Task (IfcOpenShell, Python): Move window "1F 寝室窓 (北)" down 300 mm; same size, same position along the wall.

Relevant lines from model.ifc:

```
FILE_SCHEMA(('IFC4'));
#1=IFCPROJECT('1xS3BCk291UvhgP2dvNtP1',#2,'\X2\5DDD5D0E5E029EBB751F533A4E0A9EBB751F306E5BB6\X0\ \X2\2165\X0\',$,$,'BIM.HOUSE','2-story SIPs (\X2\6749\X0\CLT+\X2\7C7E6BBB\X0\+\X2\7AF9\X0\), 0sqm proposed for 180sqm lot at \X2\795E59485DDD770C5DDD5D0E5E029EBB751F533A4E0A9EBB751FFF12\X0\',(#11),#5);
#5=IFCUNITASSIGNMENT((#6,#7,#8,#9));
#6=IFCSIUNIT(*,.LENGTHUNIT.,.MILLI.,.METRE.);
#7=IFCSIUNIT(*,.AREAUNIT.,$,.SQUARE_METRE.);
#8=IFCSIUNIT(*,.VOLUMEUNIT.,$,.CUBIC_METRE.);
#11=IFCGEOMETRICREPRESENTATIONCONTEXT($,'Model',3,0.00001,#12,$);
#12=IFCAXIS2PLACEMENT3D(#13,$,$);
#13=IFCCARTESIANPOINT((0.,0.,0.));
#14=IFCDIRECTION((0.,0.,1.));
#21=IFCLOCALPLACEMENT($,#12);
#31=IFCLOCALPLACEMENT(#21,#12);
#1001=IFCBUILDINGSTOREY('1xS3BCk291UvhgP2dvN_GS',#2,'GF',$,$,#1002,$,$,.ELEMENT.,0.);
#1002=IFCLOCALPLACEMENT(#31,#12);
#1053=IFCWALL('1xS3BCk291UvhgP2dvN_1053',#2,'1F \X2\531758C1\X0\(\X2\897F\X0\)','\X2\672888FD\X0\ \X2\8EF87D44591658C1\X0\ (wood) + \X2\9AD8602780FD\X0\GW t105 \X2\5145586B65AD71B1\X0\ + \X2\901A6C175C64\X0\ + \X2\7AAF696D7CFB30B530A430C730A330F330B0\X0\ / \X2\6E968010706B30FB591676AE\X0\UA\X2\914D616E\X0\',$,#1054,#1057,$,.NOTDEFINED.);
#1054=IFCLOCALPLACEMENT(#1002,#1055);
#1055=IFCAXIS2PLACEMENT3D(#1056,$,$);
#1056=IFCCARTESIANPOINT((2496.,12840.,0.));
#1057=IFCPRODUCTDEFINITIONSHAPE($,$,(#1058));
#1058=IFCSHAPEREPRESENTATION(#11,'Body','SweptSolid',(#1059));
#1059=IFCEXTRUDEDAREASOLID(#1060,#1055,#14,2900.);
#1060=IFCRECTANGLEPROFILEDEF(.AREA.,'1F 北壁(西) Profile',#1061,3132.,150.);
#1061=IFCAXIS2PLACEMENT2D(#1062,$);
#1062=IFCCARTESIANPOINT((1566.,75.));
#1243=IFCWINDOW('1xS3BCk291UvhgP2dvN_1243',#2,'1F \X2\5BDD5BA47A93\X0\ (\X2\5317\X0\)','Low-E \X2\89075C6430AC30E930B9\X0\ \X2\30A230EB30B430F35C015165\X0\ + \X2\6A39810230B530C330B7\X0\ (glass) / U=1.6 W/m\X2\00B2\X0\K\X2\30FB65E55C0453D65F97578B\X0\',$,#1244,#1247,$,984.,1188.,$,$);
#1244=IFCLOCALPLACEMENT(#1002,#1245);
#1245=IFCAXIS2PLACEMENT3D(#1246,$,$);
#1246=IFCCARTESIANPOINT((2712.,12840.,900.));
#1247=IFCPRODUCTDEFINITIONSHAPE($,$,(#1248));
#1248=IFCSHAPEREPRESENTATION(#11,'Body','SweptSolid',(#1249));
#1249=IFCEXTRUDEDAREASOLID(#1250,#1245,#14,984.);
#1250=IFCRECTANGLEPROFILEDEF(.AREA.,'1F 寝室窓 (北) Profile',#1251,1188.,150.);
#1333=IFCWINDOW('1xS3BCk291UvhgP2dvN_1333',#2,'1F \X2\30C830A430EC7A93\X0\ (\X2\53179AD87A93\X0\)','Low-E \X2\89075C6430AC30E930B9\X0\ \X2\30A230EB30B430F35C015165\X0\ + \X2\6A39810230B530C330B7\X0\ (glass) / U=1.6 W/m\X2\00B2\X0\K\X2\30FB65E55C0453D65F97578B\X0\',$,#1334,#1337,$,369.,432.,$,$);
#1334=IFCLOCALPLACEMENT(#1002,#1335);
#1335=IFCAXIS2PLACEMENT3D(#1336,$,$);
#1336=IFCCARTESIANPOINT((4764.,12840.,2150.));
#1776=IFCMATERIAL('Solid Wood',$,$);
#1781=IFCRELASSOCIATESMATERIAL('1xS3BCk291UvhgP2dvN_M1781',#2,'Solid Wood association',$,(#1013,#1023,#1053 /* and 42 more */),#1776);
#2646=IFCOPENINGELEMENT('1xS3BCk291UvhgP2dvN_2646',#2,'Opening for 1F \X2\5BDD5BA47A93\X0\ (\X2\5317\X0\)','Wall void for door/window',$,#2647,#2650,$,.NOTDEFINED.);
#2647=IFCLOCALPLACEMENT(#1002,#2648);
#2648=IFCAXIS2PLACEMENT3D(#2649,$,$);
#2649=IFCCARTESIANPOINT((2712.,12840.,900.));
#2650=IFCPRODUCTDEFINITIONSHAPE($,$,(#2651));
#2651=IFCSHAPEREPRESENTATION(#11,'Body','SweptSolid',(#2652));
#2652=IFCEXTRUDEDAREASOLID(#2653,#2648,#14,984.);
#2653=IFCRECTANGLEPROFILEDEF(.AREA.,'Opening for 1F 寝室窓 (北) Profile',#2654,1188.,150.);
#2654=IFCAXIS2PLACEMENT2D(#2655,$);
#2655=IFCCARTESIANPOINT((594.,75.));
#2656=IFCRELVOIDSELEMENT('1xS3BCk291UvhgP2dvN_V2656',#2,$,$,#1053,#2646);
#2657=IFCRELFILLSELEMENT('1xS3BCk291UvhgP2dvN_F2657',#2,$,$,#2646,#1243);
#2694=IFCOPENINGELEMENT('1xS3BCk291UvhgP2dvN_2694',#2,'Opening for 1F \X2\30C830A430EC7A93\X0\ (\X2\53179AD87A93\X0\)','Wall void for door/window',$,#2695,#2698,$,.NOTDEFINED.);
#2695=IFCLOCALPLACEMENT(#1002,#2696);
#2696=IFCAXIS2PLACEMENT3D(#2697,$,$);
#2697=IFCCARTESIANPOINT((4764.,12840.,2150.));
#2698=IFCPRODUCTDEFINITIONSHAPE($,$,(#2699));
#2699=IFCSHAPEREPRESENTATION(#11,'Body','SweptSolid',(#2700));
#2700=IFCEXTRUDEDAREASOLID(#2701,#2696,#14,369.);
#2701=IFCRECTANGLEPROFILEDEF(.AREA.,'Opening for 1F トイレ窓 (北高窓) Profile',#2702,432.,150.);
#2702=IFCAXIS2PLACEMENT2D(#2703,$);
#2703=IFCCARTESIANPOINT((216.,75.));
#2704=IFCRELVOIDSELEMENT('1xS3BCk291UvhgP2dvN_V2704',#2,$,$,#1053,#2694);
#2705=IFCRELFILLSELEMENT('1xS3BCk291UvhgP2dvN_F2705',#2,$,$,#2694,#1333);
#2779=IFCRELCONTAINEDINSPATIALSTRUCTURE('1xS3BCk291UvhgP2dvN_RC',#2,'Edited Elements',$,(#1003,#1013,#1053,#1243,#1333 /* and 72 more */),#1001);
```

```python
import numpy as np
import ifcopenshell
import ifcopenshell.api.geometry
import ifcopenshell.util.placement
import ifcopenshell.util.unit

model = ifcopenshell.open("model.ifc")
unit_scale = ifcopenshell.util.unit.calculate_unit_scale(model)

window = model.by_guid("1xS3BCk291UvhgP2dvN_1243")
opening = window.FillsVoids[0].RelatingOpeningElement
dz = -300.0

shift = np.array([0.0, 0.0, dz])
# The window is not placed relative to its opening, so move both.
for product in (opening, window):
    matrix = ifcopenshell.util.placement.get_local_placement(product.ObjectPlacement)
    matrix[:3, 3] += shift
    ifcopenshell.api.geometry.edit_object_placement(model, product=product, matrix=matrix, is_si=False)

print(f"moved by {dz * unit_scale:+.3f} m")

model.write("model_rev.ifc")
```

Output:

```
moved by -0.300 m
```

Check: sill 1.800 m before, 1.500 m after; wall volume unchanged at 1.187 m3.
